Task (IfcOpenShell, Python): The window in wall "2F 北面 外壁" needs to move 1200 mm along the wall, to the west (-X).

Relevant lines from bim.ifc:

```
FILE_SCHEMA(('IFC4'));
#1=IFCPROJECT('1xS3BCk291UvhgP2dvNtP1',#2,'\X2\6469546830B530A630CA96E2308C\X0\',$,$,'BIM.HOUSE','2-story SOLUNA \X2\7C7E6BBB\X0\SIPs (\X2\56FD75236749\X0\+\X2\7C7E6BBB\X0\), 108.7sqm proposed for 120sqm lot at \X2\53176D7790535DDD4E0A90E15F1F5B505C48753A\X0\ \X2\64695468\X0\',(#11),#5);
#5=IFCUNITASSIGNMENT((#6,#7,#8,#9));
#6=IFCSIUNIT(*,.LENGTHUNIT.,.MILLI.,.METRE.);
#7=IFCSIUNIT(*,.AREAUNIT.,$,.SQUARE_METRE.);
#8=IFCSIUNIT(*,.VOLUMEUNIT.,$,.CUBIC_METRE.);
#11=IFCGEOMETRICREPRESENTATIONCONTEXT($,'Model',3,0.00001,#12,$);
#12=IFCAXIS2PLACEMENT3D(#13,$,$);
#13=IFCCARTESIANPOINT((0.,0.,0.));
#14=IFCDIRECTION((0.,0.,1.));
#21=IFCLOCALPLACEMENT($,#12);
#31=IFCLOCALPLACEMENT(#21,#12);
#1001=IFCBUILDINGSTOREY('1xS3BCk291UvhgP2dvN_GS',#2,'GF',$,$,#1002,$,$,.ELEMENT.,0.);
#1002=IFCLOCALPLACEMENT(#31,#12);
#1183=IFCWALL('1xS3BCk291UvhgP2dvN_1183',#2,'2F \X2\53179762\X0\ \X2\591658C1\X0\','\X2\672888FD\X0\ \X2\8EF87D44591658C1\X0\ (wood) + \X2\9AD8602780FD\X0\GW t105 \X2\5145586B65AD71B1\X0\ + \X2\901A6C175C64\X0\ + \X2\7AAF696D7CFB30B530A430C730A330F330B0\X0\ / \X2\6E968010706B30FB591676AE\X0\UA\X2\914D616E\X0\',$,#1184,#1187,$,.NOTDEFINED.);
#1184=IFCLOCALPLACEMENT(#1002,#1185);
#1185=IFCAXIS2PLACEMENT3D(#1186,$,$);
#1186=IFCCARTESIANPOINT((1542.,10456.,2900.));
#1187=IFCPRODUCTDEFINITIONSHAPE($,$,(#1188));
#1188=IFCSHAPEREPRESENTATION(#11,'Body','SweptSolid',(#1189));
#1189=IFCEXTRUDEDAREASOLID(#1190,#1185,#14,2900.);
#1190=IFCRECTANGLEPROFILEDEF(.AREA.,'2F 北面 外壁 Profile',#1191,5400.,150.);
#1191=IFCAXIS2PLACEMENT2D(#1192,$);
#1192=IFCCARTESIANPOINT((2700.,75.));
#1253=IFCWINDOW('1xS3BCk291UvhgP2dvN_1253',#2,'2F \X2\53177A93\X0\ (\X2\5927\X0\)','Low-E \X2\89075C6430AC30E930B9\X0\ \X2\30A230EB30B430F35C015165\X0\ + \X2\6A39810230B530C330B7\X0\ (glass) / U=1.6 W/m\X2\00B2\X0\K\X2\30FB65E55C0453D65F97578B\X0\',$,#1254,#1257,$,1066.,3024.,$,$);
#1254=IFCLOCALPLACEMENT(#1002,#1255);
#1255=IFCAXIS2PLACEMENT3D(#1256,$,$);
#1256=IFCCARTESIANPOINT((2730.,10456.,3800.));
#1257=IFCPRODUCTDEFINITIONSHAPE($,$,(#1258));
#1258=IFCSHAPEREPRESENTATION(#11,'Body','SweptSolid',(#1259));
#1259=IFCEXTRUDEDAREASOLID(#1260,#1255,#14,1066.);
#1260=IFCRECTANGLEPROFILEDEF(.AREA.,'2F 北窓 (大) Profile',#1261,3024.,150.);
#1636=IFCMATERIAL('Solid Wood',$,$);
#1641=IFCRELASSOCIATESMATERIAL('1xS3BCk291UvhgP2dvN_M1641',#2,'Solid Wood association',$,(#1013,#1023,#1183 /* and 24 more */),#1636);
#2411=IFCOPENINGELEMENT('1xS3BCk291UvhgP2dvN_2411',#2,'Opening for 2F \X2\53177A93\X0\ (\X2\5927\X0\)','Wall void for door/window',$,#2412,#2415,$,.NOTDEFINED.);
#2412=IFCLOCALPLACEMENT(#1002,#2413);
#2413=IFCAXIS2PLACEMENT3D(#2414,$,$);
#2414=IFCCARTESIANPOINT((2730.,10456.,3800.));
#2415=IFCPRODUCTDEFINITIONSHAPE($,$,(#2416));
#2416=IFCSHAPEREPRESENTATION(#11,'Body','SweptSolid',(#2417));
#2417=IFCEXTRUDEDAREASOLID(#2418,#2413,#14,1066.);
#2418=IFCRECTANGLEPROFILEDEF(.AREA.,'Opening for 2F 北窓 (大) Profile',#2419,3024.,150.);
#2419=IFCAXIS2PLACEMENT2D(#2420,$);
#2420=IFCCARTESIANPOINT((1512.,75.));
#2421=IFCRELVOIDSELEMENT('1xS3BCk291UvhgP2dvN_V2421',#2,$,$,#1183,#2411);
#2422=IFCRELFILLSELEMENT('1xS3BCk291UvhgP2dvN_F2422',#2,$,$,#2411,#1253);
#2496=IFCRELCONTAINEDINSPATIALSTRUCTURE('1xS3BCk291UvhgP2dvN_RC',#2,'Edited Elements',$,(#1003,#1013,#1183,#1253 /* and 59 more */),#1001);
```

```python
import ifcopenshell
import ifcopenshell.api.geometry
import ifcopenshell.util.placement
import ifcopenshell.util.unit

model = ifcopenshell.open("bim.ifc")
unit_scale = ifcopenshell.util.unit.calculate_unit_scale(model)

window = model.by_guid("1xS3BCk291UvhgP2dvN_1253")
opening = window.FillsVoids[0].RelatingOpeningElement
wall = opening.VoidsElements[0].RelatingBuildingElement

wall_matrix = ifcopenshell.util.placement.get_local_placement(wall.ObjectPlacement)
shift = wall_matrix[:3, 0] * -1.2 / unit_scale
before = ifcopenshell.util.placement.get_local_placement(window.ObjectPlacement)[:3, 3].copy()

# The window is not placed relative to its opening, so move both.
for product in (opening, window):
    matrix = ifcopenshell.util.placement.get_local_placement(product.ObjectPlacement)
    matrix[:3, 3] += shift
    ifcopenshell.api.geometry.edit_object_placement(model, product=product, matrix=matrix, is_si=False)

after = ifcopenshell.util.placement.get_local_placement(window.ObjectPlacement)[:3, 3]
print("window moved by", (after - before).round(3) + 0.0)

model.write("bim_v2.ifc")
```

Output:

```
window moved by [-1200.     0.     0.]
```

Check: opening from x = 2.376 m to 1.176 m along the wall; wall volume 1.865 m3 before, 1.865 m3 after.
